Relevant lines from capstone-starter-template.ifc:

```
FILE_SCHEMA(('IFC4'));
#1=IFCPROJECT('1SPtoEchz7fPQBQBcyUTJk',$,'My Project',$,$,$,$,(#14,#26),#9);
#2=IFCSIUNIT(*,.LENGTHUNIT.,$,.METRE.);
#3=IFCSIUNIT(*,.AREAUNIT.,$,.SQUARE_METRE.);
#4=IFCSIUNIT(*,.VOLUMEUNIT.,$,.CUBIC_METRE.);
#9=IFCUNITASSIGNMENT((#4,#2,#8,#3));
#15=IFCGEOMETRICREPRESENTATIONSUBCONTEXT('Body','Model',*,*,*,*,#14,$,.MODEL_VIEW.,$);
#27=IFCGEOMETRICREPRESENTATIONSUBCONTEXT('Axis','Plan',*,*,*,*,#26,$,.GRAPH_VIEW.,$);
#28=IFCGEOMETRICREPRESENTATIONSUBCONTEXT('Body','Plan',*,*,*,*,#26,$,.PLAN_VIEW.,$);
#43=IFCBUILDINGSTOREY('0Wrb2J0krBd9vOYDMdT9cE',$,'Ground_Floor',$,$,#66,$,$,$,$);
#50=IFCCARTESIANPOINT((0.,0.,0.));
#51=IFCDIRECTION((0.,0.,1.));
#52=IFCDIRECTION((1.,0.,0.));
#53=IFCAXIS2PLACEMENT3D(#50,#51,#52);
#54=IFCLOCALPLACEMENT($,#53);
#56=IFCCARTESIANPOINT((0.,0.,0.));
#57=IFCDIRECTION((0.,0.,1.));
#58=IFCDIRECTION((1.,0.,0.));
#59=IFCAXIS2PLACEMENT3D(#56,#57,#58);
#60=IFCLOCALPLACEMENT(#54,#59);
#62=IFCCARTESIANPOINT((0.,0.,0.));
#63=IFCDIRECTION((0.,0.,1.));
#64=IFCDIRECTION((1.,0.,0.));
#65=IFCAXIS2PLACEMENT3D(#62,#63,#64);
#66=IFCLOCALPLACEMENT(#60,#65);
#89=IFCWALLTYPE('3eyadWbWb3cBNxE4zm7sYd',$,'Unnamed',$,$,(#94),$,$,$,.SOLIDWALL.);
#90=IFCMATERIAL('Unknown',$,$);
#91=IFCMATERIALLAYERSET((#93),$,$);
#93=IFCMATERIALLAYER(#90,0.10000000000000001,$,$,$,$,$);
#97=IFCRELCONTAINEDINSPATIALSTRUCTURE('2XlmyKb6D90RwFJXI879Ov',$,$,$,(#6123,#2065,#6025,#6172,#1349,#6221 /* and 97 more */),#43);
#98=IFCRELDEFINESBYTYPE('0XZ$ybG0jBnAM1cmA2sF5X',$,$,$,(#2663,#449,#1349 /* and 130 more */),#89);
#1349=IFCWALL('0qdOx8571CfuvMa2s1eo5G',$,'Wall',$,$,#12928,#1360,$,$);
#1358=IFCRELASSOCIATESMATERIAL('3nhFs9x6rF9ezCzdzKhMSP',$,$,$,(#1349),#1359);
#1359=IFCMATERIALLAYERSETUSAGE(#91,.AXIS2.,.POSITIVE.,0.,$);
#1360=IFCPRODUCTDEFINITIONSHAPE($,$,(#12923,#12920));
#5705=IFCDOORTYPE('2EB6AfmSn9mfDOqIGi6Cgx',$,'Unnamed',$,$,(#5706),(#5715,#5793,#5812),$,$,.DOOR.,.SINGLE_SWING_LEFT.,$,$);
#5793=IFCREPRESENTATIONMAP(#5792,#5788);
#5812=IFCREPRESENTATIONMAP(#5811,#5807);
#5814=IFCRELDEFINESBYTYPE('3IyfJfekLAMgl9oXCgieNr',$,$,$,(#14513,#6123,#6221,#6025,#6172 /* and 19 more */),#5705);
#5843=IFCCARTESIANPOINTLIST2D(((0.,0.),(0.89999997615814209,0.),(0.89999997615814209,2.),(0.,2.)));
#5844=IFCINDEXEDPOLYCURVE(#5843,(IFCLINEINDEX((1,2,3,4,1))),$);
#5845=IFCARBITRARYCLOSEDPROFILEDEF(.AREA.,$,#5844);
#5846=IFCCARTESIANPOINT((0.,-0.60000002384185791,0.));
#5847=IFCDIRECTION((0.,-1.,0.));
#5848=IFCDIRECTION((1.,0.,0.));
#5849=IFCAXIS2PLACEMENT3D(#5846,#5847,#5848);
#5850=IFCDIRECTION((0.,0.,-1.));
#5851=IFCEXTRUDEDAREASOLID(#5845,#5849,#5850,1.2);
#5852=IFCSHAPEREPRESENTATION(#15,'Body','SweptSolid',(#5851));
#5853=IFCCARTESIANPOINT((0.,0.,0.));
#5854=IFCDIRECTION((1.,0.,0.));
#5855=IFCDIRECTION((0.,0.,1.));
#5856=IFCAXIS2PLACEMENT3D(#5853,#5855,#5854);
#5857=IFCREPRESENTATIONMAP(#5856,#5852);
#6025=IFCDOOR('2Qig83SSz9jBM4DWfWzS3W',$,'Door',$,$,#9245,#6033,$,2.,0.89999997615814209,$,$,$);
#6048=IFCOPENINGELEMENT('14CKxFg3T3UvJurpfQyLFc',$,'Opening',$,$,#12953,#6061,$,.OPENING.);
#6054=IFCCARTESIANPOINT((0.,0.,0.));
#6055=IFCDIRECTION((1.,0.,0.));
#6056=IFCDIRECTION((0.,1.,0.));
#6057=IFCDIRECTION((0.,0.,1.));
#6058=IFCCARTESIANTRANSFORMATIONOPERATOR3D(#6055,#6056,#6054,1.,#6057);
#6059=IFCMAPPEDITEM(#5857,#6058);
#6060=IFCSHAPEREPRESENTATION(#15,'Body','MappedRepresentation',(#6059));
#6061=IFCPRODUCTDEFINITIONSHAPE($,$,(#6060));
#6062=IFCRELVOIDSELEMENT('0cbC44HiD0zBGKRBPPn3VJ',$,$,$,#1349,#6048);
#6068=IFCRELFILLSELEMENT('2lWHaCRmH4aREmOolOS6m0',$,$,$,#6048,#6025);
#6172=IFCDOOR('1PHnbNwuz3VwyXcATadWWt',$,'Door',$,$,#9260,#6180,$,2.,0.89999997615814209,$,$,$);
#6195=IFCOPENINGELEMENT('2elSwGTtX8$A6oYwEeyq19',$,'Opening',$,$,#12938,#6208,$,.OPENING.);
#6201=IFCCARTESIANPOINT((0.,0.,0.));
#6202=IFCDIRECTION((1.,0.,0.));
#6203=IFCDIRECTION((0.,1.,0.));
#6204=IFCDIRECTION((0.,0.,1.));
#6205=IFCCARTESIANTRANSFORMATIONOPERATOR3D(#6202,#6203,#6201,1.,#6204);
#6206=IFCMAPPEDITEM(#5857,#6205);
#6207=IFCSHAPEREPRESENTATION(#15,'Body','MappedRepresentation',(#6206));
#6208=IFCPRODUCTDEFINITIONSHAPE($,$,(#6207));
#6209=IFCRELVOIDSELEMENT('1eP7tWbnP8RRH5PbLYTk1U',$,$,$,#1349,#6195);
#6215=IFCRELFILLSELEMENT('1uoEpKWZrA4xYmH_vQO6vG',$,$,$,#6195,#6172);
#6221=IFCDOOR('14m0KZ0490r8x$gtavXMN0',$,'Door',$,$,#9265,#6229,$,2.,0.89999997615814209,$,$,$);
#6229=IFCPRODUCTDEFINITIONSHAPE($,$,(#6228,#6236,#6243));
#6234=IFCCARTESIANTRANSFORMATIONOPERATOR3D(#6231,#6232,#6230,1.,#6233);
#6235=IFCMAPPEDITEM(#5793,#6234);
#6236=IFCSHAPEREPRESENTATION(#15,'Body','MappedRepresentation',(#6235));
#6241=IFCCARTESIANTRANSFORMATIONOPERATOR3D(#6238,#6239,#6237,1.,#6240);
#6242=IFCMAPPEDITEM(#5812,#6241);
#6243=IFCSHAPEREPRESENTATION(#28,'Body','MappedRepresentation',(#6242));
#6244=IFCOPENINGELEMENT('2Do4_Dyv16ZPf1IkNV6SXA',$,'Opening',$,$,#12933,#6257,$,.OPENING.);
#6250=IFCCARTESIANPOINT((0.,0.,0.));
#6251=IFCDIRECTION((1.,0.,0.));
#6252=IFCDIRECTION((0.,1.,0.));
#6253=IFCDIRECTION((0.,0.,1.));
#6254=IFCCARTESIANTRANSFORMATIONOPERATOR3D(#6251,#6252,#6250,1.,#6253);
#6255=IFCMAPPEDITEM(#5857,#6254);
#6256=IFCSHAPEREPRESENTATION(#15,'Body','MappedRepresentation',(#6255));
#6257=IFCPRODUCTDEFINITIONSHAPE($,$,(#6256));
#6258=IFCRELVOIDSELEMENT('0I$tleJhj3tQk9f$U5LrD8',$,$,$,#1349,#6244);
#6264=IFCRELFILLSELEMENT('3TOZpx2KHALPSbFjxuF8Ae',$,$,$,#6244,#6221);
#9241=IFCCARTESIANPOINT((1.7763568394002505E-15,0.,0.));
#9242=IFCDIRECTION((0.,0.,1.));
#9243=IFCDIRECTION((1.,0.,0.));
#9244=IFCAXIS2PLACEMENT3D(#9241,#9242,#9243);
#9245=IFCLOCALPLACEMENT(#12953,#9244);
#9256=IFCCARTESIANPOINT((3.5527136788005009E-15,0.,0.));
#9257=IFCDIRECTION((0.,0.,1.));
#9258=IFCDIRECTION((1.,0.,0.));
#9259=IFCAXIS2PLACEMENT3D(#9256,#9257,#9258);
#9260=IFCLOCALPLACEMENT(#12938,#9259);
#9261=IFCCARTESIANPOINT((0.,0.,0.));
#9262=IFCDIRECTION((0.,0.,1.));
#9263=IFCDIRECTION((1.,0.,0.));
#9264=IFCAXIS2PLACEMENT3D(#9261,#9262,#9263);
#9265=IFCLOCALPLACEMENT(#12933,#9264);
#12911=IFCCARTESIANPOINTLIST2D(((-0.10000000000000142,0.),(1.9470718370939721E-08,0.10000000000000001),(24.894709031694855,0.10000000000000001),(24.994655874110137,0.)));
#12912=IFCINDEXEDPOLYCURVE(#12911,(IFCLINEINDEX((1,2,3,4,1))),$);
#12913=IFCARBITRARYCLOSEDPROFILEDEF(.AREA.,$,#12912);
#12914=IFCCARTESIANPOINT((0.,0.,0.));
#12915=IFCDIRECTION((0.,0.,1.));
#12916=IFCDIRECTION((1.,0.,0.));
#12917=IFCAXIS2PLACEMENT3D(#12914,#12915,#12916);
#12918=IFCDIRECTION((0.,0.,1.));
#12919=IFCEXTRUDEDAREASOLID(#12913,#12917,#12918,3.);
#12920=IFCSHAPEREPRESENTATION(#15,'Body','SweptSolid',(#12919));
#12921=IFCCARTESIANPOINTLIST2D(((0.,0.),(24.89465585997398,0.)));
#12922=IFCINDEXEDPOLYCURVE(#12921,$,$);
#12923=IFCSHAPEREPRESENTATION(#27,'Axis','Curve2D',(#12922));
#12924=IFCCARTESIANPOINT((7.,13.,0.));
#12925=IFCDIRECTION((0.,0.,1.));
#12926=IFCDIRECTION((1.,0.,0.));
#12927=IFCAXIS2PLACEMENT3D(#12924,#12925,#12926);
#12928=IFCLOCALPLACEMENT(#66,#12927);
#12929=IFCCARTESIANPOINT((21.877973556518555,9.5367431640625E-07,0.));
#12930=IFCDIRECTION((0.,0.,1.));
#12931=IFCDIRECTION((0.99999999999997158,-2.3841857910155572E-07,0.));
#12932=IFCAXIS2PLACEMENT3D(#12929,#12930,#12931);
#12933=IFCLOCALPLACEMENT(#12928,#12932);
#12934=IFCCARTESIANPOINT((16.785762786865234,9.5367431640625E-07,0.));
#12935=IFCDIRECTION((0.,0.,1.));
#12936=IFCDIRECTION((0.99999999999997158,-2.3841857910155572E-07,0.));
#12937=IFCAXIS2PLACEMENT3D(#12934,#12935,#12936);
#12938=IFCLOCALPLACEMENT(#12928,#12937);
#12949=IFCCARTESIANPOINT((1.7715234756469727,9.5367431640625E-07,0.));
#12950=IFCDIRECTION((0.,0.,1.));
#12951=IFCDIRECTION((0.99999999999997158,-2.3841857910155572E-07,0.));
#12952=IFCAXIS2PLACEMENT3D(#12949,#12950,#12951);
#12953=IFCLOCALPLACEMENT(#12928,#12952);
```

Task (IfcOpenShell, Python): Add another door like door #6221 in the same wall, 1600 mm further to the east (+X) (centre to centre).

```python
import ifcopenshell
import ifcopenshell.api.feature
import ifcopenshell.api.geometry
import ifcopenshell.api.root
import ifcopenshell.geom
import ifcopenshell.util.element
import ifcopenshell.util.placement
import ifcopenshell.util.shape
import ifcopenshell.util.unit

model = ifcopenshell.open("capstone-starter-template.ifc")
unit_scale = ifcopenshell.util.unit.calculate_unit_scale(model)
settings = ifcopenshell.geom.settings()


def volume(element):
    """Net volume in cubic metres, openings subtracted."""
    shape = ifcopenshell.geom.create_shape(settings, element)
    return ifcopenshell.util.shape.get_volume(shape.geometry)


door = model.by_guid("14m0KZ0490r8x$gtavXMN0")
opening = door.FillsVoids[0].RelatingOpeningElement
wall = opening.VoidsElements[0].RelatingBuildingElement
before = volume(wall)
shift = ifcopenshell.util.placement.get_local_placement(wall.ObjectPlacement)[:3, 0] * 1.6 / unit_scale

# copy_class copies the void relationship, type, container and properties, but no geometry.
new_opening = ifcopenshell.api.root.copy_class(model, product=opening)
new_opening.Representation = ifcopenshell.util.element.copy_deep(
    model, opening.Representation, exclude=["IfcGeometricRepresentationContext", "IfcRepresentationMap"]
)
new_door = ifcopenshell.api.root.copy_class(model, product=door)
new_door.Representation = ifcopenshell.util.element.copy_deep(
    model, door.Representation, exclude=["IfcGeometricRepresentationContext", "IfcRepresentationMap"]
)
ifcopenshell.api.feature.add_filling(model, opening=new_opening, element=new_door)

for old, new in ((opening, new_opening), (door, new_door)):
    matrix = ifcopenshell.util.placement.get_local_placement(old.ObjectPlacement)
    matrix[:3, 3] += shift
    ifcopenshell.api.geometry.edit_object_placement(model, product=new, matrix=matrix, is_si=False)

after = volume(wall)

print(f"wall volume {before:.3f} -> {after:.3f} m3")

model.write("capstone-starter-template_v2.ifc")
```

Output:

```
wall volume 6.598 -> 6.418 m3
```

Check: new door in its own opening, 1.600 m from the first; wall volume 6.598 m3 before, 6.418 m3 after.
